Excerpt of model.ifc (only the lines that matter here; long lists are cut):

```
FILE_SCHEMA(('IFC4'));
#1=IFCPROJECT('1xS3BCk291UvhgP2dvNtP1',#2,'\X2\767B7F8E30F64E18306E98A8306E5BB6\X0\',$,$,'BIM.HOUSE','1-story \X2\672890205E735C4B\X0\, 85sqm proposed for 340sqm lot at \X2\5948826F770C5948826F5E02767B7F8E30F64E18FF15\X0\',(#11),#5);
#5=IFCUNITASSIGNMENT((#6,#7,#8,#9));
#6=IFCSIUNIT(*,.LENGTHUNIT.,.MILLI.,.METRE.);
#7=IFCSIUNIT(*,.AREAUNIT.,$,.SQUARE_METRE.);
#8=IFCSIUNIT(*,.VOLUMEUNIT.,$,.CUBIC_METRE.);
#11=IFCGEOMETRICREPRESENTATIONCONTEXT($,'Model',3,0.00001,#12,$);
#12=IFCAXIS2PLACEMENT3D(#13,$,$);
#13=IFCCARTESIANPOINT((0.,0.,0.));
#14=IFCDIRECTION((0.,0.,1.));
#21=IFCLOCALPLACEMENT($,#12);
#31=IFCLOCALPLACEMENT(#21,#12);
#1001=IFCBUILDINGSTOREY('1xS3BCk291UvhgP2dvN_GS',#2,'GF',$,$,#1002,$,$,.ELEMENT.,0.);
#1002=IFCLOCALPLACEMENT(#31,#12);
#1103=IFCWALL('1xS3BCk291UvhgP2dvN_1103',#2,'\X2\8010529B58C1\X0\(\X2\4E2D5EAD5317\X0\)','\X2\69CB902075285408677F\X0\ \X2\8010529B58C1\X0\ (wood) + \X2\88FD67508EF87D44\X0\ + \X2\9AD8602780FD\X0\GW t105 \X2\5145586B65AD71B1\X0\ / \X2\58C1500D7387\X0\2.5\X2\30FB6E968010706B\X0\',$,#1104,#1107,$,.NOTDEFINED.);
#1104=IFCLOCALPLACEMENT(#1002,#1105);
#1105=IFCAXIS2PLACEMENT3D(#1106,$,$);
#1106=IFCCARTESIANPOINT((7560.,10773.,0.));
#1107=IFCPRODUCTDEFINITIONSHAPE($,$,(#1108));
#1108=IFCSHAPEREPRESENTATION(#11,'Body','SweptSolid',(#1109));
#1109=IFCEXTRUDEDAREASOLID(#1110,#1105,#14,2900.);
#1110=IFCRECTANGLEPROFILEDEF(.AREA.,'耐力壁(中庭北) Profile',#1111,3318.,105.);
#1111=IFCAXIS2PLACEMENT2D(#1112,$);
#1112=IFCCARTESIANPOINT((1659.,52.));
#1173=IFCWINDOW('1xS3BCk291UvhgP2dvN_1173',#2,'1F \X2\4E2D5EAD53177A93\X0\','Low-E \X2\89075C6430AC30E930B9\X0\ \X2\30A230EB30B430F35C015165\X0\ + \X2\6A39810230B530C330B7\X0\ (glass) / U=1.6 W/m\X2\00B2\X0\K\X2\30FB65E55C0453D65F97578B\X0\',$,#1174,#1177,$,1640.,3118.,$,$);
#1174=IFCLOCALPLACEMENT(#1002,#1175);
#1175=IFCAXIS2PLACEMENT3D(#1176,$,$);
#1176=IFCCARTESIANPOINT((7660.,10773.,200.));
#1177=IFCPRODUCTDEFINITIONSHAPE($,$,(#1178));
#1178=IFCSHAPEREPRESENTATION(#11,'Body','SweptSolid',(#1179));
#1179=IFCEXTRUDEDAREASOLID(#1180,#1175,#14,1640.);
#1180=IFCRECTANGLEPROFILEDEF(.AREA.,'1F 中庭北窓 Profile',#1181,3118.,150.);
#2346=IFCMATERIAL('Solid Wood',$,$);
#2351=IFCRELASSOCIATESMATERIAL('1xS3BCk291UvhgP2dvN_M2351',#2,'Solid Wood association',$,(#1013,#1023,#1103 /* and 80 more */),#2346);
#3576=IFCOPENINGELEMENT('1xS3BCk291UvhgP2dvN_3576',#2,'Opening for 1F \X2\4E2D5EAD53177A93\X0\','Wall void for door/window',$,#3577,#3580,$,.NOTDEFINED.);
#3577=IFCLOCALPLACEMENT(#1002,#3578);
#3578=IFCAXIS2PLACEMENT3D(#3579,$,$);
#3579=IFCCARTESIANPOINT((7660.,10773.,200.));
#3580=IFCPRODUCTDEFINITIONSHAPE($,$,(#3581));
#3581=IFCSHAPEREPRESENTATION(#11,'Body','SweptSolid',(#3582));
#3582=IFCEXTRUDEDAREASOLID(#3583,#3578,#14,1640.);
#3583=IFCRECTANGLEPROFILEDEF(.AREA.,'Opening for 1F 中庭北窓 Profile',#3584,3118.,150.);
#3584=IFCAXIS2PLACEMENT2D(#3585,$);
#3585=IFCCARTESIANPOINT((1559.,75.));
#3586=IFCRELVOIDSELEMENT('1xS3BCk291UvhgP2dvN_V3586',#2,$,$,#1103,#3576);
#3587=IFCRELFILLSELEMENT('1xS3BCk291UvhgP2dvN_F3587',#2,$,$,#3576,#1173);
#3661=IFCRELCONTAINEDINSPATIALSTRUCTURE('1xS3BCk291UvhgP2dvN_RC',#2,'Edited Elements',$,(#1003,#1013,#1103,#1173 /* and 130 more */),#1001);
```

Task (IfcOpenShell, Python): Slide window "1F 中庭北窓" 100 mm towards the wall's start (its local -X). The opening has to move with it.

```python
import ifcopenshell
import ifcopenshell.api.geometry
import ifcopenshell.util.placement
import ifcopenshell.util.unit

model = ifcopenshell.open("model.ifc")
unit_scale = ifcopenshell.util.unit.calculate_unit_scale(model)

window = model.by_guid("1xS3BCk291UvhgP2dvN_1173")
opening = window.FillsVoids[0].RelatingOpeningElement
wall = opening.VoidsElements[0].RelatingBuildingElement

wall_matrix = ifcopenshell.util.placement.get_local_placement(wall.ObjectPlacement)
shift = wall_matrix[:3, 0] * -0.1 / unit_scale
before = ifcopenshell.util.placement.get_local_placement(window.ObjectPlacement)[:3, 3].copy()

# The window is not placed relative to its opening, so move both.
for product in (opening, window):
    matrix = ifcopenshell.util.placement.get_local_placement(product.ObjectPlacement)
    matrix[:3, 3] += shift
    ifcopenshell.api.geometry.edit_object_placement(model, product=product, matrix=matrix, is_si=False)

after = ifcopenshell.util.placement.get_local_placement(window.ObjectPlacement)[:3, 3]
print("window moved by", (after - before).round(3) + 0.0)

model.write("model_updated.ifc")
```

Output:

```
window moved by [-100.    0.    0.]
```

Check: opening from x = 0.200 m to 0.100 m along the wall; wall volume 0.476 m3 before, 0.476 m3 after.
